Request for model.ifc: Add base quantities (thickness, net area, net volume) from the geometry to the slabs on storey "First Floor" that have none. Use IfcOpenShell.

First a look at what the model holds.

```python
import ifcopenshell
import ifcopenshell.util.element
import ifcopenshell.util.unit

model = ifcopenshell.open("model.ifc")
print(model.schema)
for unit_type in ("LENGTHUNIT", "AREAUNIT", "VOLUMEUNIT"):
    print(unit_type, ifcopenshell.util.unit.calculate_unit_scale(model, unit_type))
storey = next(s for s in model.by_type("IfcBuildingStorey") if s.Name == "First Floor")
slabs = [e for e in ifcopenshell.util.element.get_decomposition(storey) if e.is_a("IfcSlab")]
for e in sorted(slabs, key=lambda e: e.id()):
    print(e.id(), e.is_a(), e.Name, list(ifcopenshell.util.element.get_psets(e, qtos_only=True)), sep=" | ")
```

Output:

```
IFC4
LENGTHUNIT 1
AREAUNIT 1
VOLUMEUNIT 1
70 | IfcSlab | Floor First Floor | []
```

```python
import ifcopenshell
import ifcopenshell.api.pset
import ifcopenshell.geom
import ifcopenshell.util.element
import ifcopenshell.util.shape
import ifcopenshell.util.unit

model = ifcopenshell.open("model.ifc")
unit_scale = ifcopenshell.util.unit.calculate_unit_scale(model)
area_scale = ifcopenshell.util.unit.calculate_unit_scale(model, "AREAUNIT")
volume_scale = ifcopenshell.util.unit.calculate_unit_scale(model, "VOLUMEUNIT")
settings = ifcopenshell.geom.settings()

storey = next(s for s in model.by_type("IfcBuildingStorey") if s.Name == "First Floor")
slabs = [e for e in ifcopenshell.util.element.get_decomposition(storey) if e.is_a("IfcSlab")]

for e in sorted(slabs, key=lambda e: e.id()):
    if ifcopenshell.util.element.get_psets(e, qtos_only=True, should_inherit=False):
        continue
    # Geometry comes back in metres, in the element's own axes.
    shape = ifcopenshell.geom.create_shape(settings, e)
    values = {
        "Width": ifcopenshell.util.shape.get_z(shape.geometry) / unit_scale,
        "NetArea": ifcopenshell.util.shape.get_footprint_area(shape.geometry) / area_scale,
        "NetVolume": ifcopenshell.util.shape.get_volume(shape.geometry) / volume_scale,
    }
    qto = ifcopenshell.api.pset.add_qto(model, product=e, name="Qto_SlabBaseQuantities")
    ifcopenshell.api.pset.edit_qto(model, qto=qto, properties=values)
    print(e.id(), {k: round(v, 3) for k, v in values.items()})

model.write("model_updated.ifc")
```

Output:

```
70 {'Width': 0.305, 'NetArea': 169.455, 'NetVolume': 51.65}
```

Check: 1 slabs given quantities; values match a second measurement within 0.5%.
